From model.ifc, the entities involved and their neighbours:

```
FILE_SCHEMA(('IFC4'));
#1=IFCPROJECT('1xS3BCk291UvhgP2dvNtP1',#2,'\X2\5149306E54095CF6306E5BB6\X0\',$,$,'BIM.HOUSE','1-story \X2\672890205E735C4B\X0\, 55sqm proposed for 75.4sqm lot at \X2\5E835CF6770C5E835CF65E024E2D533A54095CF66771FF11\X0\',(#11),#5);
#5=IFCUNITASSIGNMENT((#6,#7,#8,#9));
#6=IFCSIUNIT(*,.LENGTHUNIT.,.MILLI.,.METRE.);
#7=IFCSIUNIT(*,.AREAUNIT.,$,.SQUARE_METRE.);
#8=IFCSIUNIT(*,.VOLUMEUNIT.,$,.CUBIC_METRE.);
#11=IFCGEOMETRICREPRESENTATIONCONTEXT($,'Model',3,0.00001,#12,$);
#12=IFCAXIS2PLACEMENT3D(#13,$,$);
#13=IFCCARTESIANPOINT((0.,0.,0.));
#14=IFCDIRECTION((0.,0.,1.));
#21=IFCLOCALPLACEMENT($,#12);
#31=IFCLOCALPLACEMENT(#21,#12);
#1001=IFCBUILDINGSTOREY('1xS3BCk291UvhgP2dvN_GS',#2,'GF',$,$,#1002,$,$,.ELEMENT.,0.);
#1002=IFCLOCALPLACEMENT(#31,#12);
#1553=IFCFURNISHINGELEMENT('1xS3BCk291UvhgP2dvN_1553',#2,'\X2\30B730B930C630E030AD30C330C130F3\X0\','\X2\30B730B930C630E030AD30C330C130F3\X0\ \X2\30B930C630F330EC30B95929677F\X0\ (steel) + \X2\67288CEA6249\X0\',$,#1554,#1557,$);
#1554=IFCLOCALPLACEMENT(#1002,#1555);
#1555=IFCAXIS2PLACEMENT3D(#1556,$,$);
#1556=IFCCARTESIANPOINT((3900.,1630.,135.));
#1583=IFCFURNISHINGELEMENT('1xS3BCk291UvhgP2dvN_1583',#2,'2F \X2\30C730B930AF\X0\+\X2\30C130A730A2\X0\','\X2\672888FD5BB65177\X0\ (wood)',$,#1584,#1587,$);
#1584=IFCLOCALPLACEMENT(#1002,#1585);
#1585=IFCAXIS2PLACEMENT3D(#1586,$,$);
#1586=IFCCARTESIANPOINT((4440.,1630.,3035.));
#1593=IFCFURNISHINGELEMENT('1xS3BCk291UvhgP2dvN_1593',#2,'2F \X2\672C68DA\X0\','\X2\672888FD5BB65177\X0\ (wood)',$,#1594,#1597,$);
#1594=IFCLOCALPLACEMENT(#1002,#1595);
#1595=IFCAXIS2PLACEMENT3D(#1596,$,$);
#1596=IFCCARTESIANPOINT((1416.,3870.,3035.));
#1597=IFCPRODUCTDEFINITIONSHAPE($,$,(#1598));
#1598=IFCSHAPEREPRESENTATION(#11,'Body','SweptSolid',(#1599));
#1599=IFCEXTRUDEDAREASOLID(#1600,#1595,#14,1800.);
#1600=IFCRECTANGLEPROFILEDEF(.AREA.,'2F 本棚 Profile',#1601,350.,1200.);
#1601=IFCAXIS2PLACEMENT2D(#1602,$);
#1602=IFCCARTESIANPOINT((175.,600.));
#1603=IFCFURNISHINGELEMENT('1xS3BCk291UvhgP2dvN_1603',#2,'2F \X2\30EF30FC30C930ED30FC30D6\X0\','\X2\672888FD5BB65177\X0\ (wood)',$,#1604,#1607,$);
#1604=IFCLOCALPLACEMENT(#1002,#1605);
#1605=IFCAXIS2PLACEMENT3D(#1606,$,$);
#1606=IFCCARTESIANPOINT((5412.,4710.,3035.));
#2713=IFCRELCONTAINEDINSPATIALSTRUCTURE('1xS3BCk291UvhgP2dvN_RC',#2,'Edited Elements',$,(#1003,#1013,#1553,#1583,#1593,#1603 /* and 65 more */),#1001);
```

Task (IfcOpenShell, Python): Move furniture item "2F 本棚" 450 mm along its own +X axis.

```python
import ifcopenshell
import ifcopenshell.api.geometry
import ifcopenshell.util.placement
import ifcopenshell.util.unit

model = ifcopenshell.open("model.ifc")
unit_scale = ifcopenshell.util.unit.calculate_unit_scale(model)

item = model.by_id(1593)
matrix = ifcopenshell.util.placement.get_local_placement(item.ObjectPlacement)
matrix[:3, 3] += matrix[:3, 0] * 0.45 / unit_scale
ifcopenshell.api.geometry.edit_object_placement(model, product=item, matrix=matrix, is_si=False)

print(ifcopenshell.util.placement.get_local_placement(item.ObjectPlacement).round(3) + 0.0)

model.write("model_v2.ifc")
```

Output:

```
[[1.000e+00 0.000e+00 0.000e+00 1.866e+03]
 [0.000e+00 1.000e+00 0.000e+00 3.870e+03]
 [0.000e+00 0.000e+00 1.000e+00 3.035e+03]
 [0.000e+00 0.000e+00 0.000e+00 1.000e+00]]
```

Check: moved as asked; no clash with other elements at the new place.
